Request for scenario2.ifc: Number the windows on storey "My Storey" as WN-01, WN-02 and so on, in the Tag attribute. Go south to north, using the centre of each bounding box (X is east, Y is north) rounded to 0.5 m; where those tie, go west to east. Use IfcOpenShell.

First a look at what the model holds.

```python
import ifcopenshell
import ifcopenshell.util.element
import ifcopenshell.util.placement

model = ifcopenshell.open("scenario2.ifc")
print(model.schema)
storey = next(s for s in model.by_type("IfcBuildingStorey") if s.Name == "My Storey")
windows = [e for e in ifcopenshell.util.element.get_decomposition(storey) if e.is_a("IfcWindow")]
for e in sorted(windows, key=lambda e: e.id()):
    origin = ifcopenshell.util.placement.get_local_placement(e.ObjectPlacement)[:3, 3]
    print(e.id(), e.Tag, e.Name, origin.round(2) + 0.0, sep=" | ")
```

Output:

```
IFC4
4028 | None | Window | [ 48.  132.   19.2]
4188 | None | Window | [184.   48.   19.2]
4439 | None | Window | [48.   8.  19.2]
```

```python
import ifcopenshell
import ifcopenshell.geom
import ifcopenshell.util.element
import ifcopenshell.util.shape

model = ifcopenshell.open("scenario2.ifc")
settings = ifcopenshell.geom.settings()
settings.set("use-world-coords", True)


def centre(element):
    shape = ifcopenshell.geom.create_shape(settings, element)
    return ifcopenshell.util.shape.get_bbox_centroid(shape.geometry)


storey = next(s for s in model.by_type("IfcBuildingStorey") if s.Name == "My Storey")
windows = [e for e in ifcopenshell.util.element.get_decomposition(storey) if e.is_a("IfcWindow")]

# Insertion points can sit at a corner or the storey origin, so sort by the geometry (in metres).
centres = {e: centre(e) for e in windows}
windows.sort(key=lambda e: (round(centres[e][1] / 0.5), centres[e][0]))

for i, e in enumerate(windows, start=1):
    number = f"WN-{i:02d}"
    e.Tag = number
    print(e.id(), number)

model.write("scenario2-out.ifc")
```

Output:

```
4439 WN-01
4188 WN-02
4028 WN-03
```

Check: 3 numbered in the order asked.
